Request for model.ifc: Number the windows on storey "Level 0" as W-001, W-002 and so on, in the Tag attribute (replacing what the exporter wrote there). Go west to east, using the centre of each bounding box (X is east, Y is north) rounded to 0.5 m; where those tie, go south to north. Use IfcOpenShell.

First a look at what the model holds.

```python
import ifcopenshell
import ifcopenshell.util.element
import ifcopenshell.util.placement

model = ifcopenshell.open("model.ifc")
print(model.schema)
storey = next(s for s in model.by_type("IfcBuildingStorey") if s.Name == "Level 0")
windows = [e for e in ifcopenshell.util.element.get_decomposition(storey) if e.is_a("IfcWindow")]
for e in sorted(windows, key=lambda e: e.id()):
    origin = ifcopenshell.util.placement.get_local_placement(e.ObjectPlacement)[:3, 3]
    print(e.id(), e.Tag, e.Name, origin.round(2) + 0.0, sep=" | ")
```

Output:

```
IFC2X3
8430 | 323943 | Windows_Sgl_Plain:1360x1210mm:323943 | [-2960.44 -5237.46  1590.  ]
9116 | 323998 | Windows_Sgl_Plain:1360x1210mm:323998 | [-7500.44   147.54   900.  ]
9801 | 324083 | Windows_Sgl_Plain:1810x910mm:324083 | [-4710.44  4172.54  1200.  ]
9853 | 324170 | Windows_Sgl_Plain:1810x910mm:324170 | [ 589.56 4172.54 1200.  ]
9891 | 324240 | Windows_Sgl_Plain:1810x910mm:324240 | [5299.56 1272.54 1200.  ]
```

```python
import ifcopenshell
import ifcopenshell.geom
import ifcopenshell.util.element
import ifcopenshell.util.shape

model = ifcopenshell.open("model.ifc")
settings = ifcopenshell.geom.settings()
settings.set("use-world-coords", True)


def centre(element):
    shape = ifcopenshell.geom.create_shape(settings, element)
    return ifcopenshell.util.shape.get_bbox_centroid(shape.geometry)


storey = next(s for s in model.by_type("IfcBuildingStorey") if s.Name == "Level 0")
windows = [e for e in ifcopenshell.util.element.get_decomposition(storey) if e.is_a("IfcWindow")]

# Insertion points can sit at a corner or the storey origin, so sort by the geometry (in metres).
centres = {e: centre(e) for e in windows}
windows.sort(key=lambda e: (round(centres[e][0] / 0.5), centres[e][1]))

for i, e in enumerate(windows, start=1):
    number = f"W-0{i:02d}"
    e.Tag = number
    print(e.id(), number)

model.write("model-out.ifc")
```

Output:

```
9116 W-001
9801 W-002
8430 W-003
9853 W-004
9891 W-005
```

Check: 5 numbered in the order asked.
